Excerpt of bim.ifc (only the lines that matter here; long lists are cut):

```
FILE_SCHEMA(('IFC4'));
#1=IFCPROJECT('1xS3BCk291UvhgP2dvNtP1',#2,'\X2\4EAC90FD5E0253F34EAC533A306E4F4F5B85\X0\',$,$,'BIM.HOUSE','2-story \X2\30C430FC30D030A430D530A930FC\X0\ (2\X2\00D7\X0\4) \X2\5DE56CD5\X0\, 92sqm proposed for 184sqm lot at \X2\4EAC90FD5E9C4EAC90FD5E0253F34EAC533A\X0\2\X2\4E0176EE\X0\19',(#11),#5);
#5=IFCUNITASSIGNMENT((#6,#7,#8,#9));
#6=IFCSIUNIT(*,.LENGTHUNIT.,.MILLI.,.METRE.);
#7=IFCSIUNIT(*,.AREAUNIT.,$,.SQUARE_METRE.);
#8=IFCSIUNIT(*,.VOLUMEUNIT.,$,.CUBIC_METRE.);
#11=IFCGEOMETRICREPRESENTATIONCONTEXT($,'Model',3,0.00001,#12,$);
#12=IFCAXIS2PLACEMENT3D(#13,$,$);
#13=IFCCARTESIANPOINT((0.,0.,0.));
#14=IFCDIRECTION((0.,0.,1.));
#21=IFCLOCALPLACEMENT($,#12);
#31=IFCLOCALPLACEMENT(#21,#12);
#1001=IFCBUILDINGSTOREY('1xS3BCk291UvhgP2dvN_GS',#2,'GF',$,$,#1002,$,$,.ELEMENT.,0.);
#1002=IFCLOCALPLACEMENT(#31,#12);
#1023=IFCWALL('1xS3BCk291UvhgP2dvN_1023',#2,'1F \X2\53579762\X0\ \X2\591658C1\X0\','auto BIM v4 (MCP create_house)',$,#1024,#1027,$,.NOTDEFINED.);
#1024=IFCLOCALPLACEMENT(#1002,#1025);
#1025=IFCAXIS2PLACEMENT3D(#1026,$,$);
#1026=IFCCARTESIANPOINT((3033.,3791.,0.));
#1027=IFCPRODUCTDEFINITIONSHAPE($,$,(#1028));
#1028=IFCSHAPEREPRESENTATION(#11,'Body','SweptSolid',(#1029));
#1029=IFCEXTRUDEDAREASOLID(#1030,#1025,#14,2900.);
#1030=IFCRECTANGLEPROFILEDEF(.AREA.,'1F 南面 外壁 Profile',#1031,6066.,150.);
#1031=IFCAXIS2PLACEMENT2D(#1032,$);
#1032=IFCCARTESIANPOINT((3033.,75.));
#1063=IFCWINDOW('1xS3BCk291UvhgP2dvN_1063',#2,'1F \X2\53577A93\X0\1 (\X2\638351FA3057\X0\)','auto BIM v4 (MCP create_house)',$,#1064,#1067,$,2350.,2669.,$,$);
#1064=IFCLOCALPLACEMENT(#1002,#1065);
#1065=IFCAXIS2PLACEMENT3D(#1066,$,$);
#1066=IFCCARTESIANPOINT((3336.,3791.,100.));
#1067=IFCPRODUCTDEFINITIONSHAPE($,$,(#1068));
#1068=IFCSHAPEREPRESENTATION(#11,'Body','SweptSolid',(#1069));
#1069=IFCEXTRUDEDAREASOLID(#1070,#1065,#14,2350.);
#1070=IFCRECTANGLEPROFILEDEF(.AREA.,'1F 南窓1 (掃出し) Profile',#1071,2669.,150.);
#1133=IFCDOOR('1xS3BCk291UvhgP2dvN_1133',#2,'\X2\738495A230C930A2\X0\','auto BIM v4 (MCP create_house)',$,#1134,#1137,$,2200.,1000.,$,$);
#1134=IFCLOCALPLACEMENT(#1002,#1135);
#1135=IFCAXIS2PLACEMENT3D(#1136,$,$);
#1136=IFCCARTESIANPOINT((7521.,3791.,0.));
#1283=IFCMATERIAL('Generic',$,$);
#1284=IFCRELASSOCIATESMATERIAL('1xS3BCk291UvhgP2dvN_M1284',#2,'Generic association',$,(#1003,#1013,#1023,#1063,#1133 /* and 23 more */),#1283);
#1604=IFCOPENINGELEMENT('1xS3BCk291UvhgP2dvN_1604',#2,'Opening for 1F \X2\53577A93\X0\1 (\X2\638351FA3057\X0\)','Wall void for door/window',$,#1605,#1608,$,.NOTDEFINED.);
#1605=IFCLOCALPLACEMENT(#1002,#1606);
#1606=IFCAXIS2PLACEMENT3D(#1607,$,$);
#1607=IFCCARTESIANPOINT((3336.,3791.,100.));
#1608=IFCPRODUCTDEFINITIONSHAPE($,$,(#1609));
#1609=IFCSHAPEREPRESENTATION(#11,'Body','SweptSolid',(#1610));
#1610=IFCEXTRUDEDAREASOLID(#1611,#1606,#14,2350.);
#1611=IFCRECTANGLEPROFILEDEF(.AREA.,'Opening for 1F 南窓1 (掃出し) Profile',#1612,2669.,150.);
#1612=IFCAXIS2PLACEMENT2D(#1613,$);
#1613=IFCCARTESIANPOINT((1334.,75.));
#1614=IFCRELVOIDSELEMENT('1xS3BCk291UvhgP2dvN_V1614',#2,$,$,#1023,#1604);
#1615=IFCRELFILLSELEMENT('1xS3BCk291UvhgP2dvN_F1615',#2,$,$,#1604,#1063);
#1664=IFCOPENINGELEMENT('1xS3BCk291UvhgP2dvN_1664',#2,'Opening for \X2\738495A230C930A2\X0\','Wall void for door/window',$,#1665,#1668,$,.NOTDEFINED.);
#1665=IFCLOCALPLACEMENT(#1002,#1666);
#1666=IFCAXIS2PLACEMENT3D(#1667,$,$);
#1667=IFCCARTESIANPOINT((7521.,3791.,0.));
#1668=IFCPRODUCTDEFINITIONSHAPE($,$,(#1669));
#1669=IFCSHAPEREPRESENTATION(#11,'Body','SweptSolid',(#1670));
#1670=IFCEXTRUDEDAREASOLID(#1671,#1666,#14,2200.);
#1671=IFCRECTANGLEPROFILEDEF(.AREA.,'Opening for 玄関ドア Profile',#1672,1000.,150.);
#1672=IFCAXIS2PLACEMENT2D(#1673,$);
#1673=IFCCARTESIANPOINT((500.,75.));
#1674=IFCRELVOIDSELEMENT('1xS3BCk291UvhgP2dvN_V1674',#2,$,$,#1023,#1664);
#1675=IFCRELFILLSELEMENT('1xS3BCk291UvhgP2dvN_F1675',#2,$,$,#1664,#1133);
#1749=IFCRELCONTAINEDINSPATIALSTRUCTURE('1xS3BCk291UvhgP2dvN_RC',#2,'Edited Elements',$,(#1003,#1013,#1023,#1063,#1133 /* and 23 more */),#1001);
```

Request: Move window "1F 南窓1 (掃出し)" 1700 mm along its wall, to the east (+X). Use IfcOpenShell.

```python
import ifcopenshell
import ifcopenshell.api.geometry
import ifcopenshell.util.placement
import ifcopenshell.util.unit

model = ifcopenshell.open("bim.ifc")
unit_scale = ifcopenshell.util.unit.calculate_unit_scale(model)

window = model.by_guid("1xS3BCk291UvhgP2dvN_1063")
opening = window.FillsVoids[0].RelatingOpeningElement
wall = opening.VoidsElements[0].RelatingBuildingElement

wall_matrix = ifcopenshell.util.placement.get_local_placement(wall.ObjectPlacement)
shift = wall_matrix[:3, 0] * 1.7 / unit_scale
before = ifcopenshell.util.placement.get_local_placement(window.ObjectPlacement)[:3, 3].copy()

# The window is not placed relative to its opening, so move both.
for product in (opening, window):
    matrix = ifcopenshell.util.placement.get_local_placement(product.ObjectPlacement)
    matrix[:3, 3] += shift
    ifcopenshell.api.geometry.edit_object_placement(model, product=product, matrix=matrix, is_si=False)

after = ifcopenshell.util.placement.get_local_placement(window.ObjectPlacement)[:3, 3]
print("window moved by", (after - before).round(3) + 0.0)

model.write("bim_v2.ifc")
```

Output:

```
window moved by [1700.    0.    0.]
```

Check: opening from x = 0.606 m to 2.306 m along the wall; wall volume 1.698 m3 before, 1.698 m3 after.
